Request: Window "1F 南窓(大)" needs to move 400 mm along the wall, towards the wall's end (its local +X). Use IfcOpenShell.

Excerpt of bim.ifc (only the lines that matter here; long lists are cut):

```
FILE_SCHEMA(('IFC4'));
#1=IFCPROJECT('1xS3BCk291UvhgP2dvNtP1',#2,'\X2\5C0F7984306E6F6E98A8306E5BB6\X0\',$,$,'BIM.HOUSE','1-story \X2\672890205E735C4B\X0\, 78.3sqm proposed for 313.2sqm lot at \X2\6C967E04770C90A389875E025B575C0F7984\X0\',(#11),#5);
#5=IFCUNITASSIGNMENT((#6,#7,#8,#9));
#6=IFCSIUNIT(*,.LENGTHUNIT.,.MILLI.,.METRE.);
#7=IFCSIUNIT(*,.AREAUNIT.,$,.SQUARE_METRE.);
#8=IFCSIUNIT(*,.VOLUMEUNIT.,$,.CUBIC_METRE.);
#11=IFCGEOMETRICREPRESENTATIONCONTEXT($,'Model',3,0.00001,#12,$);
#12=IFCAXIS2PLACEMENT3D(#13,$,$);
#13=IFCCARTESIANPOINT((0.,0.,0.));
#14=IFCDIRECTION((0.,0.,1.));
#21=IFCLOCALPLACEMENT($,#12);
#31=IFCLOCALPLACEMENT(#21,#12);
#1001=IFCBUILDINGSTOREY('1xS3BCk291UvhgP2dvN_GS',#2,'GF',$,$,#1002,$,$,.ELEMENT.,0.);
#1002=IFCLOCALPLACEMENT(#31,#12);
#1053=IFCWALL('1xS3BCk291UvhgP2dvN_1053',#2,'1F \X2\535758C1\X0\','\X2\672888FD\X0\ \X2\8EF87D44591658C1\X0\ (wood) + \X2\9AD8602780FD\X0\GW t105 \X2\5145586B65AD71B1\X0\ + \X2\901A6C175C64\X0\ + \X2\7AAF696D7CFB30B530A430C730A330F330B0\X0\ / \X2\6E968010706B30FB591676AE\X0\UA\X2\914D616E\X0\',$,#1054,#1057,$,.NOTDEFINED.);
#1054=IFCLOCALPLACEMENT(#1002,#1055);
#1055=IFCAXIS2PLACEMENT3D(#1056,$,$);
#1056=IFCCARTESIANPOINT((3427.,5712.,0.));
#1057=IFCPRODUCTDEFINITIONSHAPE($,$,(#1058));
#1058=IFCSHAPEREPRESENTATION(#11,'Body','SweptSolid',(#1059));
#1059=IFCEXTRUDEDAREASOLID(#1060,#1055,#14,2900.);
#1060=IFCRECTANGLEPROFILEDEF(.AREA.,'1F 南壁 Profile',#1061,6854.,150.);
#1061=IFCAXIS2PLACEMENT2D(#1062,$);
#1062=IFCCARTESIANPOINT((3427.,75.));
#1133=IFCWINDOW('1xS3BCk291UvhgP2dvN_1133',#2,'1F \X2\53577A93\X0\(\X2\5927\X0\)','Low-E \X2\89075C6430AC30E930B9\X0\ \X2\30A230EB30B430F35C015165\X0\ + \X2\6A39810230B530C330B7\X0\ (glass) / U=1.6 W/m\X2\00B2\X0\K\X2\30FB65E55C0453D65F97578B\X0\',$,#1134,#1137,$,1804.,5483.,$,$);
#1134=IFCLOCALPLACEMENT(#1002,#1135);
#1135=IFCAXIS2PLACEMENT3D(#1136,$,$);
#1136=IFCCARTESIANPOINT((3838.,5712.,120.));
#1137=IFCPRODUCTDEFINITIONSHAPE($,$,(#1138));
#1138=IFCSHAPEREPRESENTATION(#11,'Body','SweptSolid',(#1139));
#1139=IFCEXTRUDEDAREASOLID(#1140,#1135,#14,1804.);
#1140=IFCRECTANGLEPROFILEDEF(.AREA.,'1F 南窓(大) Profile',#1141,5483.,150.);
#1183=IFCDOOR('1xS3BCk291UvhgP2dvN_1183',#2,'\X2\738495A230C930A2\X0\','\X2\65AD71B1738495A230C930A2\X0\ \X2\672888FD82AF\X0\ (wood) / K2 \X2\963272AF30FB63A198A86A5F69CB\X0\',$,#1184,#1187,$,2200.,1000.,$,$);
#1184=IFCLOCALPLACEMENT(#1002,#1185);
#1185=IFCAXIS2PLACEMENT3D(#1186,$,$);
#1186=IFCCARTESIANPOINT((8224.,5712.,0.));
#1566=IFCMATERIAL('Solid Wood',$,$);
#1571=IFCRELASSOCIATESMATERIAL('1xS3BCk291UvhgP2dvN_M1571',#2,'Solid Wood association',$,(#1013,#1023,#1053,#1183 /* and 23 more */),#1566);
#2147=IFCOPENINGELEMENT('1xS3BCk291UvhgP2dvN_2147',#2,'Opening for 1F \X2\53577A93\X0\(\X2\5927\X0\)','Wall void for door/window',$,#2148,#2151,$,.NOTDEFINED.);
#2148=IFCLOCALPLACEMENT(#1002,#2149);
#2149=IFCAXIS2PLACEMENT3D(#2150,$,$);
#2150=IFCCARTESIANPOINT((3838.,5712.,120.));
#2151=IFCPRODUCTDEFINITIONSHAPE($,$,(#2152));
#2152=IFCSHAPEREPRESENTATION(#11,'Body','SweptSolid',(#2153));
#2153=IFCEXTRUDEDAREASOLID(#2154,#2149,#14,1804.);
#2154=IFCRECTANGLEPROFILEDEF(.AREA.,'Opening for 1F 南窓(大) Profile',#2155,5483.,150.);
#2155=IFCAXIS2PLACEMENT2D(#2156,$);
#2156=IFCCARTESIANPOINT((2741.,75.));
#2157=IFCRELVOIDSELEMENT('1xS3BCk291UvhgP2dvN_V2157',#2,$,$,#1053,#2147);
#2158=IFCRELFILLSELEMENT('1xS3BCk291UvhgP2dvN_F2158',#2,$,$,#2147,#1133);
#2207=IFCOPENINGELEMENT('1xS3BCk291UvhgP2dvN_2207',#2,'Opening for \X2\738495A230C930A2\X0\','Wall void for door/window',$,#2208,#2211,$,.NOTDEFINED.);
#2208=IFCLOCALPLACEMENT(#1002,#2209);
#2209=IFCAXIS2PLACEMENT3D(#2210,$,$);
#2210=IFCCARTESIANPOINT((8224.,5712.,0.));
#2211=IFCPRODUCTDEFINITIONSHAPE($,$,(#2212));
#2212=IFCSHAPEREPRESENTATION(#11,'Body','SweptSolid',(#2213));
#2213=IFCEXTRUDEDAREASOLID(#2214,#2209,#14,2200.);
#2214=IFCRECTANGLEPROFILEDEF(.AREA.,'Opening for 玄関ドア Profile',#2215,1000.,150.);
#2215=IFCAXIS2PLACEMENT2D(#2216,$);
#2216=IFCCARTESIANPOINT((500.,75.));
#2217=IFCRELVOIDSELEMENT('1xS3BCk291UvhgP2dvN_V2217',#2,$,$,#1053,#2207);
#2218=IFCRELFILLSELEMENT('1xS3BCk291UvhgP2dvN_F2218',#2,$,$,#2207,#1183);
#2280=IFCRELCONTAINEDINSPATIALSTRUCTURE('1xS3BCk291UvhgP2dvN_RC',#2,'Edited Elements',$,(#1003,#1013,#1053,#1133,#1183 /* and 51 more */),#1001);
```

```python
import ifcopenshell
import ifcopenshell.api.geometry
import ifcopenshell.util.placement
import ifcopenshell.util.unit

model = ifcopenshell.open("bim.ifc")
unit_scale = ifcopenshell.util.unit.calculate_unit_scale(model)

window = model.by_guid("1xS3BCk291UvhgP2dvN_1133")
opening = window.FillsVoids[0].RelatingOpeningElement
wall = opening.VoidsElements[0].RelatingBuildingElement

wall_matrix = ifcopenshell.util.placement.get_local_placement(wall.ObjectPlacement)
shift = wall_matrix[:3, 0] * 0.4 / unit_scale
before = ifcopenshell.util.placement.get_local_placement(window.ObjectPlacement)[:3, 3].copy()

# The window is not placed relative to its opening, so move both.
for product in (opening, window):
    matrix = ifcopenshell.util.placement.get_local_placement(product.ObjectPlacement)
    matrix[:3, 3] += shift
    ifcopenshell.api.geometry.edit_object_placement(model, product=product, matrix=matrix, is_si=False)

after = ifcopenshell.util.placement.get_local_placement(window.ObjectPlacement)[:3, 3]
print("window moved by", (after - before).round(3) + 0.0)

model.write("bim_v2.ifc")
```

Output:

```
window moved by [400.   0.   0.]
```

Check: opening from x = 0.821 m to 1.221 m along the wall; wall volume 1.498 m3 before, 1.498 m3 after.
